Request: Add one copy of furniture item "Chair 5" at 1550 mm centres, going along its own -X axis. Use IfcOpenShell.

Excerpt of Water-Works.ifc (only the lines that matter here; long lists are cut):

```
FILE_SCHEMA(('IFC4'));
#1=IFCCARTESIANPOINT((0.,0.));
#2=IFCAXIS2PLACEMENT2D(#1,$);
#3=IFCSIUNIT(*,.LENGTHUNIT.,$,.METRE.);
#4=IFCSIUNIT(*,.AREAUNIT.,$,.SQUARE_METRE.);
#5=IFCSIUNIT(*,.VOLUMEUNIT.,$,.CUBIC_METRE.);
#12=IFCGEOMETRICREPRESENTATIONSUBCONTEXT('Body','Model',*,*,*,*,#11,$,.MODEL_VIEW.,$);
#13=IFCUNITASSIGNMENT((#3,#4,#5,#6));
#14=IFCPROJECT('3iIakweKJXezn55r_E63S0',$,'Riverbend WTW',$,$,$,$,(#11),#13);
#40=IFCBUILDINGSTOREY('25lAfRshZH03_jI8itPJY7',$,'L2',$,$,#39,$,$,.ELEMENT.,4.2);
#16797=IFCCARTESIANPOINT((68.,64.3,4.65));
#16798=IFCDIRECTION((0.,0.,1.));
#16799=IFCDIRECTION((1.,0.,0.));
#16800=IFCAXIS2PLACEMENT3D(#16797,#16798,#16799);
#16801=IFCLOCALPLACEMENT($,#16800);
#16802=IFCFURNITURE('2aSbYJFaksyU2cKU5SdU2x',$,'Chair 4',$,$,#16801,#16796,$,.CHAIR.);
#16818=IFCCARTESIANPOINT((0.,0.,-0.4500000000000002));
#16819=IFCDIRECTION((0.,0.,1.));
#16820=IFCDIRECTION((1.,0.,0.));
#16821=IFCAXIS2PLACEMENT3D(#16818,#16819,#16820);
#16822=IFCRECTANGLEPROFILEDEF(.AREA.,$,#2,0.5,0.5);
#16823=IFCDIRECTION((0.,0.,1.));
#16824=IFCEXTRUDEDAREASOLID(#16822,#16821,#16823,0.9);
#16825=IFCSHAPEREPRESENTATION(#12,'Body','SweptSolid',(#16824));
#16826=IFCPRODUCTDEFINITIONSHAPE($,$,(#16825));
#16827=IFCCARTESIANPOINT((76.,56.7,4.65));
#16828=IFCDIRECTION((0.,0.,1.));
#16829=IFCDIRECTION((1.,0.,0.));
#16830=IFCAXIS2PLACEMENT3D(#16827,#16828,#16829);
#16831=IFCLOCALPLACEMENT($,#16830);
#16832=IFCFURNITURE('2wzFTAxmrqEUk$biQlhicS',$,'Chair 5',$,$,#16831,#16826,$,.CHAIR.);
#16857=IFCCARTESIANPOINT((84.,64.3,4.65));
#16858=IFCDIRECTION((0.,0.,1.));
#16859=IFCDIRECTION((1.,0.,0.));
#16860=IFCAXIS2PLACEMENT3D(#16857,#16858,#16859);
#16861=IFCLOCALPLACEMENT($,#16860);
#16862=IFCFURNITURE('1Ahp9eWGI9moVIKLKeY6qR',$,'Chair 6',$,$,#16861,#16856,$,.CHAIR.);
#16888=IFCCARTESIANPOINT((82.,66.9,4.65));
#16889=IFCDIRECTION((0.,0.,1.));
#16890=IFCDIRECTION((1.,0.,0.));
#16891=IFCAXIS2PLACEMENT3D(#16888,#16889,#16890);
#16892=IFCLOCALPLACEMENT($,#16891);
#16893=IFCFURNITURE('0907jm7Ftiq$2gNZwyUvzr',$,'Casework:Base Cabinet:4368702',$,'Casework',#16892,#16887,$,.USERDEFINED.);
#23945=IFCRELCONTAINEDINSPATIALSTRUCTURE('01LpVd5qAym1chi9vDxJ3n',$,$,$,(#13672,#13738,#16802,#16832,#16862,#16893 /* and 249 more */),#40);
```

```python
import ifcopenshell
import ifcopenshell.api.geometry
import ifcopenshell.api.root
import ifcopenshell.util.element
import ifcopenshell.util.placement
import ifcopenshell.util.unit

model = ifcopenshell.open("Water-Works.ifc")
unit_scale = ifcopenshell.util.unit.calculate_unit_scale(model)

source = model.by_guid("2wzFTAxmrqEUk$biQlhicS")
base = ifcopenshell.util.placement.get_local_placement(source.ObjectPlacement)
step = -base[:3, 0] * 1.55 / unit_scale

for i in range(1, 2):
    copy = ifcopenshell.api.root.copy_class(model, product=source)
    copy.Representation = ifcopenshell.util.element.copy_deep(
        model, source.Representation, exclude=["IfcGeometricRepresentationContext", "IfcRepresentationMap"]
    )
    matrix = base.copy()
    matrix[:3, 3] += i * step
    print("added at", matrix[:3, 3].round(3) + 0.0)
    ifcopenshell.api.geometry.edit_object_placement(model, product=copy, matrix=matrix, is_si=False)

model.write("Water-Works_updated.ifc")
```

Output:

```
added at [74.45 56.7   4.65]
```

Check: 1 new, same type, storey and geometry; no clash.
